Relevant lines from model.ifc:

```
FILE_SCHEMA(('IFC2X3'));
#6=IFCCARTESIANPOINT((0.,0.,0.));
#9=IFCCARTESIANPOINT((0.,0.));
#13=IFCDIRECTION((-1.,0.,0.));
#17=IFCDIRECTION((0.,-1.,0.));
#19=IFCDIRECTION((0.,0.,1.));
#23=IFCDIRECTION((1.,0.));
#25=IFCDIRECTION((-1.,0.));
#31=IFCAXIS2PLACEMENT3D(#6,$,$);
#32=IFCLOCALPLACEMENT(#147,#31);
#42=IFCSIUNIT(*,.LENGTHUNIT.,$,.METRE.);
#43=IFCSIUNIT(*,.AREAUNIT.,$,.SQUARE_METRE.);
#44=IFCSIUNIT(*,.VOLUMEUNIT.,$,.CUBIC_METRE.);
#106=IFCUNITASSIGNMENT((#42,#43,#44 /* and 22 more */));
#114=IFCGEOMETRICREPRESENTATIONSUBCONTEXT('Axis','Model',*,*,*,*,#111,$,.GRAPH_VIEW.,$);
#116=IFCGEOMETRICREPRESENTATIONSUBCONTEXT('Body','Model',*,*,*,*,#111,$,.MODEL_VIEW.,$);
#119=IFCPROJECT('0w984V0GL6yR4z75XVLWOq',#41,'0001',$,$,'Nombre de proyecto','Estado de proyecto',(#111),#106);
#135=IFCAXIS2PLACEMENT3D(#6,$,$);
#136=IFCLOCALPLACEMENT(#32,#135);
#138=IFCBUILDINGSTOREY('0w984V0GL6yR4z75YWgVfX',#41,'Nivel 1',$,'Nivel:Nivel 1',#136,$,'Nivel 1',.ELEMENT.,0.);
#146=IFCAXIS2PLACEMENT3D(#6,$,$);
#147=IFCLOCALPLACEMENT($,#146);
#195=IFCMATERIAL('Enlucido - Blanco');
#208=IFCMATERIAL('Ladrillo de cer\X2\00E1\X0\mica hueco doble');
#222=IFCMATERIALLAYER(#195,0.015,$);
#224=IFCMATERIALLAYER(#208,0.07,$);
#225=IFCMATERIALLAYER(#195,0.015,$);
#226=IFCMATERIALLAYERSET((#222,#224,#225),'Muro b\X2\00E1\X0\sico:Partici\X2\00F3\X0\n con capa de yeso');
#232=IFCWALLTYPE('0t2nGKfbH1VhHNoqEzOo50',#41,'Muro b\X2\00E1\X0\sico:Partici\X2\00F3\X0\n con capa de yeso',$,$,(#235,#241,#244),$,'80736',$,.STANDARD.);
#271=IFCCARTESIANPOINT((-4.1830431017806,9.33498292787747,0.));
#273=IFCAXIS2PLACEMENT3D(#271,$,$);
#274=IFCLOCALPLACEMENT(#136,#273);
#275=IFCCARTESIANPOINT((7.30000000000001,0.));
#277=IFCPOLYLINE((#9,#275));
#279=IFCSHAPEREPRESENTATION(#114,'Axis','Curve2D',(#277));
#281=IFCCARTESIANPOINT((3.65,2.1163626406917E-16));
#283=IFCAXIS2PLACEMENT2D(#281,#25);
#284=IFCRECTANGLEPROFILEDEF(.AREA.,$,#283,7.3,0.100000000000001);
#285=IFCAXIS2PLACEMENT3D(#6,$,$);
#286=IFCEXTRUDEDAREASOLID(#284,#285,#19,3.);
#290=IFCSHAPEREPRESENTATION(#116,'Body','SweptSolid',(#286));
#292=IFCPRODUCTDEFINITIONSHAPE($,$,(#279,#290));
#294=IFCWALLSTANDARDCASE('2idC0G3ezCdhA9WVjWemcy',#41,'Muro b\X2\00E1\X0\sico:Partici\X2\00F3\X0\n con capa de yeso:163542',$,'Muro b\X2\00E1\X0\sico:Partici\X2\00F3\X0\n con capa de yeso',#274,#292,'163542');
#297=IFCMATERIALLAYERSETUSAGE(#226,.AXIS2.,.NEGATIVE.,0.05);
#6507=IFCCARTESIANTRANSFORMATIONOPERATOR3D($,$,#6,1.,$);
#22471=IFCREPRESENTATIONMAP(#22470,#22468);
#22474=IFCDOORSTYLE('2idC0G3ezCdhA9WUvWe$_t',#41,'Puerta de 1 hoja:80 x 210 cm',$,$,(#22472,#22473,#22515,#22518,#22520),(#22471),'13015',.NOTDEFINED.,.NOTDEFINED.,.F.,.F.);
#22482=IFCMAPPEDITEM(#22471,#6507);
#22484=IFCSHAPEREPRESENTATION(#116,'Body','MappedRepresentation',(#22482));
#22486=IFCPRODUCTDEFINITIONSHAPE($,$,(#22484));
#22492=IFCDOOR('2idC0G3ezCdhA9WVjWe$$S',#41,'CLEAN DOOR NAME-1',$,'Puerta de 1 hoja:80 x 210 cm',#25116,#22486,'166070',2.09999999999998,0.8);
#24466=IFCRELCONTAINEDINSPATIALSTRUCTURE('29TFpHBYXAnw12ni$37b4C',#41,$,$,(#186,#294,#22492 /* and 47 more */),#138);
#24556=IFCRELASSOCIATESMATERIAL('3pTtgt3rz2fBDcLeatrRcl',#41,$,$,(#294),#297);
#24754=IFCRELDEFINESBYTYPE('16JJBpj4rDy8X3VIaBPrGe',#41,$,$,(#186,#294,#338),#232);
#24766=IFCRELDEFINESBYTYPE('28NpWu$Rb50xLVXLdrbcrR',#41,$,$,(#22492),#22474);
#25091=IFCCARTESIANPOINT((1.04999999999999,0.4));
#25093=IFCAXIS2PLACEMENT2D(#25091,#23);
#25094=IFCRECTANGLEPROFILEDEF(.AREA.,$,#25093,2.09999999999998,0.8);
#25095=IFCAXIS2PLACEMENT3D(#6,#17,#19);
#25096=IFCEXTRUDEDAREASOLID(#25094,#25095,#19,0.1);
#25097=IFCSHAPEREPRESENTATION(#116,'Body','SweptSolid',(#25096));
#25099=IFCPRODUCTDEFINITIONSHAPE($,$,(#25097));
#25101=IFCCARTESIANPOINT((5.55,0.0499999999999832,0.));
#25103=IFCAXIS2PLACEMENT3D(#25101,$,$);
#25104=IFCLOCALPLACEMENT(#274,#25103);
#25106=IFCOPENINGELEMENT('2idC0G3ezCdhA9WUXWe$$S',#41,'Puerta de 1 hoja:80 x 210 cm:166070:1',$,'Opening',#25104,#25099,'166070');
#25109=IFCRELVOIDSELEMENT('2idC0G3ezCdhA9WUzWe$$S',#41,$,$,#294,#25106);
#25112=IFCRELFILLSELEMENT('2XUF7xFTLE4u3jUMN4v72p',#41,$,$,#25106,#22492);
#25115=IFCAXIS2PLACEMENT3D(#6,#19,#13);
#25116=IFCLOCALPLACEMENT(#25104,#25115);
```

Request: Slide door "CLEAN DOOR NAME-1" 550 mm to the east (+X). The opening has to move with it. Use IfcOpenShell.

```python
import ifcopenshell
import ifcopenshell.api.geometry
import ifcopenshell.util.placement

model = ifcopenshell.open("model.ifc")

door = model.by_guid("2idC0G3ezCdhA9WVjWe$$S")
opening = door.FillsVoids[0].RelatingOpeningElement
wall = opening.VoidsElements[0].RelatingBuildingElement

wall_matrix = ifcopenshell.util.placement.get_local_placement(wall.ObjectPlacement)
shift = wall_matrix[:3, 0] * 0.55
before = ifcopenshell.util.placement.get_local_placement(door.ObjectPlacement)[:3, 3].copy()

# The door is placed relative to its opening, so it follows when the opening moves.
matrix = ifcopenshell.util.placement.get_local_placement(opening.ObjectPlacement)
matrix[:3, 3] += shift
ifcopenshell.api.geometry.edit_object_placement(
    model, product=opening, matrix=matrix, is_si=False, should_transform_children=True
)

after = ifcopenshell.util.placement.get_local_placement(door.ObjectPlacement)[:3, 3]
print("door moved by", (after - before).round(3) + 0.0)

model.write("model_v2.ifc")
```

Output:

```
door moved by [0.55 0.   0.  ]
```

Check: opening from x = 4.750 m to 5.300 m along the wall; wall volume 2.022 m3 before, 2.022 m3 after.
